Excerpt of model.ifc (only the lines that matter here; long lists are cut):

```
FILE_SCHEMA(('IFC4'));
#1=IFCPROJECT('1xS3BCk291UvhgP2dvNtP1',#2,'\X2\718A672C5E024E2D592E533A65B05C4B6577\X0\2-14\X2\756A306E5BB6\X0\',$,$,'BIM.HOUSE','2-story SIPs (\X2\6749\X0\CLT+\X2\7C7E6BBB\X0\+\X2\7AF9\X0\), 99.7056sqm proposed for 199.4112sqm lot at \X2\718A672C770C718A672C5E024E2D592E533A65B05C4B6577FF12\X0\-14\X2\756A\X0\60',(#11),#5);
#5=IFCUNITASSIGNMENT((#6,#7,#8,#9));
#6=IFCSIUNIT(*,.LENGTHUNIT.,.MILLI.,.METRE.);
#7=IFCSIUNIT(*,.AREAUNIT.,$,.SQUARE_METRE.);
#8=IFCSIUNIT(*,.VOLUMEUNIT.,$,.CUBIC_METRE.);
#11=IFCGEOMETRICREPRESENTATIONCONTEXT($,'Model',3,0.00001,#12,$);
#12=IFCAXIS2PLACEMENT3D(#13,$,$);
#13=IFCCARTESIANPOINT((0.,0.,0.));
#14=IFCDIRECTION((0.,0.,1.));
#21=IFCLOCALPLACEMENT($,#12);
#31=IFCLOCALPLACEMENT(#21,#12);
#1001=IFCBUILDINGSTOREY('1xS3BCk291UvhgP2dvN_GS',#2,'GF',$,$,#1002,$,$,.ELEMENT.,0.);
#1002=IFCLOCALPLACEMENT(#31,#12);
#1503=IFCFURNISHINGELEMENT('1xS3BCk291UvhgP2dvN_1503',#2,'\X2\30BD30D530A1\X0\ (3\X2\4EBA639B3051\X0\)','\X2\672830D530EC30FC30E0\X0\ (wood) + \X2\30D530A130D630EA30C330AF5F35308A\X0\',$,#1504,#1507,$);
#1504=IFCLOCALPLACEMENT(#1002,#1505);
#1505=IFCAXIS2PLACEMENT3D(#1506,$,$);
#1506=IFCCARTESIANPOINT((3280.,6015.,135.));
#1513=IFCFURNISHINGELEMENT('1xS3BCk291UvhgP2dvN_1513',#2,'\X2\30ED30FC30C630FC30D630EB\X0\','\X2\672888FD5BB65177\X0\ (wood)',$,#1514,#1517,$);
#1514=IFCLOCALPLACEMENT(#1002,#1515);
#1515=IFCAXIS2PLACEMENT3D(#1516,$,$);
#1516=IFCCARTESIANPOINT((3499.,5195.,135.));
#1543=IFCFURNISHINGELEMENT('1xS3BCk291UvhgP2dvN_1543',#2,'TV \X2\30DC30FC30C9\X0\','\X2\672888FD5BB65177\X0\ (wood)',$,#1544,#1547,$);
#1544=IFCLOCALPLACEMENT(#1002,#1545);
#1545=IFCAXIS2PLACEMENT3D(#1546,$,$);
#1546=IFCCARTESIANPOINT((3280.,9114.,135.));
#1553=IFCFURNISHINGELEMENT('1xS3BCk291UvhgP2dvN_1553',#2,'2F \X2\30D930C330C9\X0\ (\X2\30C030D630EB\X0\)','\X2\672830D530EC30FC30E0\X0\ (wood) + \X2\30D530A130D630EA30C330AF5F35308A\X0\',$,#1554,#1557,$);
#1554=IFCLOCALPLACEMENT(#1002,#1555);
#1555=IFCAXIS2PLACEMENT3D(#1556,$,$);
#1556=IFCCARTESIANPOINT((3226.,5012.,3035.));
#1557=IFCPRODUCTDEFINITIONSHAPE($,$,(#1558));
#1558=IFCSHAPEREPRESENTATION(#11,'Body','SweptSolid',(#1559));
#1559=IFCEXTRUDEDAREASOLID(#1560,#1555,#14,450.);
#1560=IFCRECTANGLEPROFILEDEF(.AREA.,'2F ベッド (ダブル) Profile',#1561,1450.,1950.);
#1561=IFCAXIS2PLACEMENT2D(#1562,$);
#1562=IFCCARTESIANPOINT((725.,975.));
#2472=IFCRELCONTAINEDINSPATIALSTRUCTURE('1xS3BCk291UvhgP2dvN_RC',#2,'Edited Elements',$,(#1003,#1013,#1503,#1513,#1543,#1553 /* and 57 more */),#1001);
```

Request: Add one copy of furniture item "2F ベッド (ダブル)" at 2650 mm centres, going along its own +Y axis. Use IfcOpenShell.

```python
import ifcopenshell
import ifcopenshell.api.geometry
import ifcopenshell.api.root
import ifcopenshell.util.element
import ifcopenshell.util.placement
import ifcopenshell.util.unit

model = ifcopenshell.open("model.ifc")
unit_scale = ifcopenshell.util.unit.calculate_unit_scale(model)


def reuse_history(source, copy):
    """copy_class also copies each property set's owner history, people and application; keep the originals."""
    for rel in copy.IsDefinedBy:
        if rel.is_a("IfcRelDefinesByProperties") and (history := rel.RelatingPropertyDefinition.OwnerHistory):
            rel.RelatingPropertyDefinition.OwnerHistory = source.OwnerHistory
            ifcopenshell.util.element.remove_deep2(model, history)


source = model.by_id(1553)
base = ifcopenshell.util.placement.get_local_placement(source.ObjectPlacement)
step = base[:3, 1] * 2.65 / unit_scale

for i in range(1, 2):
    copy = ifcopenshell.api.root.copy_class(model, product=source)
    copy.Representation = ifcopenshell.util.element.copy_deep(
        model, source.Representation, exclude=["IfcGeometricRepresentationContext", "IfcRepresentationMap"]
    )
    reuse_history(source, copy)
    matrix = base.copy()
    matrix[:3, 3] += i * step
    print("added at", matrix[:3, 3].round(3) + 0.0)
    ifcopenshell.api.geometry.edit_object_placement(model, product=copy, matrix=matrix, is_si=False)

model.write("model_updated.ifc")
```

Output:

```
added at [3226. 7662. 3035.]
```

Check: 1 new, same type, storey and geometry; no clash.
